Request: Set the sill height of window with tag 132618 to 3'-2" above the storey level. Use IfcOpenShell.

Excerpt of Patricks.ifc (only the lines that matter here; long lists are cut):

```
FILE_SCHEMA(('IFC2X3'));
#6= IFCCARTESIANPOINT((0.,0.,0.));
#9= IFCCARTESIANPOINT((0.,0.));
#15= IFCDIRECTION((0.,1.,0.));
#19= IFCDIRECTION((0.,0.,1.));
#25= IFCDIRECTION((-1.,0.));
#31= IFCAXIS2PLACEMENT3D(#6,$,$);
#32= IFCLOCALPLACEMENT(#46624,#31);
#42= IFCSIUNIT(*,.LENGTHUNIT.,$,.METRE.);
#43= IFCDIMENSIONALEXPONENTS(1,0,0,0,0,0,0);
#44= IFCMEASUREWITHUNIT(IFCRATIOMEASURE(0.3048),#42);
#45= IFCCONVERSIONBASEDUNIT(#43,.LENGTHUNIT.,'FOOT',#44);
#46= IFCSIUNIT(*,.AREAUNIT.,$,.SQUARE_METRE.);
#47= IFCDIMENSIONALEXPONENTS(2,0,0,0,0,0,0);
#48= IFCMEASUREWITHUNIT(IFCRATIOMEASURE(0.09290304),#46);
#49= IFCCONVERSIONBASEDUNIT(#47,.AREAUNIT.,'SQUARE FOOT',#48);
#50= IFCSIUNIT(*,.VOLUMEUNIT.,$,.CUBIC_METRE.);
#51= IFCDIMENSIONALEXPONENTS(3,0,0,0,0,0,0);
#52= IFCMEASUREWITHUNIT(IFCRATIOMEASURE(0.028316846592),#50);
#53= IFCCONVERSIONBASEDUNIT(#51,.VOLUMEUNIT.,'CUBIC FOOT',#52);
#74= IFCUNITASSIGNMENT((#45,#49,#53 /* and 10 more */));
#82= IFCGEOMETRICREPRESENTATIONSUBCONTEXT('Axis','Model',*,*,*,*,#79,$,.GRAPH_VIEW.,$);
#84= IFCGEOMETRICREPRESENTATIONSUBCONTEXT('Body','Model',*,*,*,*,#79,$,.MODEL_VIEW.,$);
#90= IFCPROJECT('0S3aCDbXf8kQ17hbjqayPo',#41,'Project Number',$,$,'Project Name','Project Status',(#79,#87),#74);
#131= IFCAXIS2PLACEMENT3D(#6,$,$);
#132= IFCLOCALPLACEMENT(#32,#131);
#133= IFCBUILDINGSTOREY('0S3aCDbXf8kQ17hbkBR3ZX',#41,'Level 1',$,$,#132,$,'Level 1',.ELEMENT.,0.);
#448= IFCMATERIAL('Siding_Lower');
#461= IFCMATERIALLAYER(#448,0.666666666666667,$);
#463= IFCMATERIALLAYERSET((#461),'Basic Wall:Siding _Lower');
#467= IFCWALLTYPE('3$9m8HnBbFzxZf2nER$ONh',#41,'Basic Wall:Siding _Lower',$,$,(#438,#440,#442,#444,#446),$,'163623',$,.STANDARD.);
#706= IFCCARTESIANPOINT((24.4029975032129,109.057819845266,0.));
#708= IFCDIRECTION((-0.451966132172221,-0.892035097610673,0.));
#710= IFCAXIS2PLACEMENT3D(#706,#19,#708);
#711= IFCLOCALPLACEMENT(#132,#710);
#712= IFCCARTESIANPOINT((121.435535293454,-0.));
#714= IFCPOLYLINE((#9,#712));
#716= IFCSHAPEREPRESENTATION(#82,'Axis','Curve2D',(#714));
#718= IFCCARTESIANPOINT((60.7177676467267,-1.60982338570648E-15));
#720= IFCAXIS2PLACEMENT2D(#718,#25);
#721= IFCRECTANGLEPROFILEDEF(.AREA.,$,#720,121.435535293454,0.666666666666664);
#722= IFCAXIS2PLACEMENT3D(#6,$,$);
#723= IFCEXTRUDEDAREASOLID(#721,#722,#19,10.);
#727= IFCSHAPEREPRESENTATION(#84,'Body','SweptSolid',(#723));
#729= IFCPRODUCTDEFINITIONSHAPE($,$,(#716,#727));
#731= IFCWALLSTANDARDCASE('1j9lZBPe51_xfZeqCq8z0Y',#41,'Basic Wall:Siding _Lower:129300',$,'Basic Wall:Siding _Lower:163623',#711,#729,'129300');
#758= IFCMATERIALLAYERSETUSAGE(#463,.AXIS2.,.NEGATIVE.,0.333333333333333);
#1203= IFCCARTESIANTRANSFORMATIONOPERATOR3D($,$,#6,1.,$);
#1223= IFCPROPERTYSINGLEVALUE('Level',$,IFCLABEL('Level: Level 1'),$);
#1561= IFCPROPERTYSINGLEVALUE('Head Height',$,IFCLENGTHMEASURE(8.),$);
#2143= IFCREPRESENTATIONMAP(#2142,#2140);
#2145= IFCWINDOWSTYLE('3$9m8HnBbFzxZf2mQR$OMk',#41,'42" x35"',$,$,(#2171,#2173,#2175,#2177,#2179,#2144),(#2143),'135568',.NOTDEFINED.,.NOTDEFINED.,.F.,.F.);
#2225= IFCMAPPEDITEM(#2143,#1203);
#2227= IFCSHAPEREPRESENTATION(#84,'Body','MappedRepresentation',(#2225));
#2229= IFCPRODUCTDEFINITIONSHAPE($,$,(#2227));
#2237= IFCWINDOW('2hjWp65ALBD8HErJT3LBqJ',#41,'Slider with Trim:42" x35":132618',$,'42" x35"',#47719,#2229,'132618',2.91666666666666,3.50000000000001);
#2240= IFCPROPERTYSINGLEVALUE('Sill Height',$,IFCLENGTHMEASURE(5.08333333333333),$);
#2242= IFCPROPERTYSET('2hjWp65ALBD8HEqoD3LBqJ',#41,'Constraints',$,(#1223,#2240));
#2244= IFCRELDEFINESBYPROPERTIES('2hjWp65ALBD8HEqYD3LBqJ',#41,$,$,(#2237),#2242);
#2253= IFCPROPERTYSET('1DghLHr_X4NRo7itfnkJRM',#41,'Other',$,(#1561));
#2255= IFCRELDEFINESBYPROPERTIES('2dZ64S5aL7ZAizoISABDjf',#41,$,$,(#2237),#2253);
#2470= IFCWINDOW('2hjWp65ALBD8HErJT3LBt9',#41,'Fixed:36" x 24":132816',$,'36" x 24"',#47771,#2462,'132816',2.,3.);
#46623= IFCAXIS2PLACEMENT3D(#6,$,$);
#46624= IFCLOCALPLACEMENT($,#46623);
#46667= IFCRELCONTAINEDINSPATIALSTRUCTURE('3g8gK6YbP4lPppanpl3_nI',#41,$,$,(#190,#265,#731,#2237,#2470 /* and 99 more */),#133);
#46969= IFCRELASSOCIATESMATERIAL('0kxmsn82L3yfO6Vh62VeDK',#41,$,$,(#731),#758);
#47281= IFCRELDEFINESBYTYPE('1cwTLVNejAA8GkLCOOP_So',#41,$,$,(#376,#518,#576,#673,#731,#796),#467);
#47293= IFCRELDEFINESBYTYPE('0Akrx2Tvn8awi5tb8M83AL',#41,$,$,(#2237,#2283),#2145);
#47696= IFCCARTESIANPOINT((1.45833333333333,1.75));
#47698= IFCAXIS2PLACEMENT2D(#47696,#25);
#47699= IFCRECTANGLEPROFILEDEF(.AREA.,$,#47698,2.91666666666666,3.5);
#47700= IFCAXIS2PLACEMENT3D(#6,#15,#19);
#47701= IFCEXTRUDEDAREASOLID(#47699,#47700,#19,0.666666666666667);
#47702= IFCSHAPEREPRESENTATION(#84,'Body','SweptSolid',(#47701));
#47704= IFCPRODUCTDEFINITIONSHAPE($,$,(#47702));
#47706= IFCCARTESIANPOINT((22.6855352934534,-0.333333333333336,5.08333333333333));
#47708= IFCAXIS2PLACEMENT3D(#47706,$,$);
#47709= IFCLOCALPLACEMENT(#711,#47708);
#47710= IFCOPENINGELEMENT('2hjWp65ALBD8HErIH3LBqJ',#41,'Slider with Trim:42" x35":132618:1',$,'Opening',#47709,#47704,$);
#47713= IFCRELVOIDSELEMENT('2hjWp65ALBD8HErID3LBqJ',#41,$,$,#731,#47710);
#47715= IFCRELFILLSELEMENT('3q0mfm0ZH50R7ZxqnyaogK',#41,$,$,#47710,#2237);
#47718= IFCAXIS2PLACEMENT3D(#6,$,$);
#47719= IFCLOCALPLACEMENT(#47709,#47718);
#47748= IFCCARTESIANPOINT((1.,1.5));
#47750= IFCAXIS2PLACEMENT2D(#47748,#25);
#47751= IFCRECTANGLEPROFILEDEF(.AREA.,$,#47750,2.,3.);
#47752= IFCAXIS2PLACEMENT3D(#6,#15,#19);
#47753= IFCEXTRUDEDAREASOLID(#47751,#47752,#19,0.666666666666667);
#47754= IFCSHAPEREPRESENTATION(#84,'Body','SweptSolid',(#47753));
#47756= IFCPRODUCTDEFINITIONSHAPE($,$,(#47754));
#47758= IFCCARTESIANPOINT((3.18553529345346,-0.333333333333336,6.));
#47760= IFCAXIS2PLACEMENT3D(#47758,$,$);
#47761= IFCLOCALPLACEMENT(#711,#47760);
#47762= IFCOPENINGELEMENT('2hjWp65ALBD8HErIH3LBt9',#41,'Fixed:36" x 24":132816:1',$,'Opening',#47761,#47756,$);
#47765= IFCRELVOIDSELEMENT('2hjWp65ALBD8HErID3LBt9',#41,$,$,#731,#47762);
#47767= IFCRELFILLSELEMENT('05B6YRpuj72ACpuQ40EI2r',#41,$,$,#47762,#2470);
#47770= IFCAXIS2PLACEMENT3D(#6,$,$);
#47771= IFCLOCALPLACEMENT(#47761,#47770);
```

```python
import numpy as np
import ifcopenshell
import ifcopenshell.api.geometry
import ifcopenshell.api.pset
import ifcopenshell.geom
import ifcopenshell.util.element
import ifcopenshell.util.placement
import ifcopenshell.util.shape
import ifcopenshell.util.unit

model = ifcopenshell.open("Patricks.ifc")
unit_scale = ifcopenshell.util.unit.calculate_unit_scale(model)

window = model.by_guid("2hjWp65ALBD8HErJT3LBqJ")
opening = window.FillsVoids[0].RelatingOpeningElement
storey = ifcopenshell.util.element.get_container(window, ifc_class="IfcBuildingStorey")
level = ifcopenshell.util.placement.get_local_placement(storey.ObjectPlacement)[2, 3]

# The opening's origin need not be at the sill, so measure its lowest point.
shape = ifcopenshell.geom.create_shape(ifcopenshell.geom.settings(), opening)
bottom = ifcopenshell.util.shape.get_shape_bottom_elevation(shape, shape.geometry) / unit_scale
dz = level + 38 * 0.0254 / unit_scale - bottom

shift = np.array([0.0, 0.0, dz])
# The window is placed relative to its opening, so it follows when the opening moves.
matrix = ifcopenshell.util.placement.get_local_placement(opening.ObjectPlacement)
matrix[:3, 3] += shift
ifcopenshell.api.geometry.edit_object_placement(
    model, product=opening, matrix=matrix, is_si=False, should_transform_children=True
)

# Keep the stored heights in step.
pset = model.by_id(ifcopenshell.util.element.get_pset(window, "Constraints", should_inherit=False)["id"])
ifcopenshell.api.pset.edit_pset(model, pset=pset, properties={
    "Sill Height": model.create_entity("IfcLengthMeasure", ifcopenshell.util.element.get_pset(window, "Constraints", "Sill Height") + dz),
})
pset = model.by_id(ifcopenshell.util.element.get_pset(window, "Other", should_inherit=False)["id"])
ifcopenshell.api.pset.edit_pset(model, pset=pset, properties={
    "Head Height": model.create_entity("IfcLengthMeasure", ifcopenshell.util.element.get_pset(window, "Other", "Head Height") + dz),
})

print(f"moved by {dz * unit_scale:+.3f} m")

model.write("Patricks_rev.ifc")
```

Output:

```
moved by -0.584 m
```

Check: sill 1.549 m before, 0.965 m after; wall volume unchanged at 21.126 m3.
